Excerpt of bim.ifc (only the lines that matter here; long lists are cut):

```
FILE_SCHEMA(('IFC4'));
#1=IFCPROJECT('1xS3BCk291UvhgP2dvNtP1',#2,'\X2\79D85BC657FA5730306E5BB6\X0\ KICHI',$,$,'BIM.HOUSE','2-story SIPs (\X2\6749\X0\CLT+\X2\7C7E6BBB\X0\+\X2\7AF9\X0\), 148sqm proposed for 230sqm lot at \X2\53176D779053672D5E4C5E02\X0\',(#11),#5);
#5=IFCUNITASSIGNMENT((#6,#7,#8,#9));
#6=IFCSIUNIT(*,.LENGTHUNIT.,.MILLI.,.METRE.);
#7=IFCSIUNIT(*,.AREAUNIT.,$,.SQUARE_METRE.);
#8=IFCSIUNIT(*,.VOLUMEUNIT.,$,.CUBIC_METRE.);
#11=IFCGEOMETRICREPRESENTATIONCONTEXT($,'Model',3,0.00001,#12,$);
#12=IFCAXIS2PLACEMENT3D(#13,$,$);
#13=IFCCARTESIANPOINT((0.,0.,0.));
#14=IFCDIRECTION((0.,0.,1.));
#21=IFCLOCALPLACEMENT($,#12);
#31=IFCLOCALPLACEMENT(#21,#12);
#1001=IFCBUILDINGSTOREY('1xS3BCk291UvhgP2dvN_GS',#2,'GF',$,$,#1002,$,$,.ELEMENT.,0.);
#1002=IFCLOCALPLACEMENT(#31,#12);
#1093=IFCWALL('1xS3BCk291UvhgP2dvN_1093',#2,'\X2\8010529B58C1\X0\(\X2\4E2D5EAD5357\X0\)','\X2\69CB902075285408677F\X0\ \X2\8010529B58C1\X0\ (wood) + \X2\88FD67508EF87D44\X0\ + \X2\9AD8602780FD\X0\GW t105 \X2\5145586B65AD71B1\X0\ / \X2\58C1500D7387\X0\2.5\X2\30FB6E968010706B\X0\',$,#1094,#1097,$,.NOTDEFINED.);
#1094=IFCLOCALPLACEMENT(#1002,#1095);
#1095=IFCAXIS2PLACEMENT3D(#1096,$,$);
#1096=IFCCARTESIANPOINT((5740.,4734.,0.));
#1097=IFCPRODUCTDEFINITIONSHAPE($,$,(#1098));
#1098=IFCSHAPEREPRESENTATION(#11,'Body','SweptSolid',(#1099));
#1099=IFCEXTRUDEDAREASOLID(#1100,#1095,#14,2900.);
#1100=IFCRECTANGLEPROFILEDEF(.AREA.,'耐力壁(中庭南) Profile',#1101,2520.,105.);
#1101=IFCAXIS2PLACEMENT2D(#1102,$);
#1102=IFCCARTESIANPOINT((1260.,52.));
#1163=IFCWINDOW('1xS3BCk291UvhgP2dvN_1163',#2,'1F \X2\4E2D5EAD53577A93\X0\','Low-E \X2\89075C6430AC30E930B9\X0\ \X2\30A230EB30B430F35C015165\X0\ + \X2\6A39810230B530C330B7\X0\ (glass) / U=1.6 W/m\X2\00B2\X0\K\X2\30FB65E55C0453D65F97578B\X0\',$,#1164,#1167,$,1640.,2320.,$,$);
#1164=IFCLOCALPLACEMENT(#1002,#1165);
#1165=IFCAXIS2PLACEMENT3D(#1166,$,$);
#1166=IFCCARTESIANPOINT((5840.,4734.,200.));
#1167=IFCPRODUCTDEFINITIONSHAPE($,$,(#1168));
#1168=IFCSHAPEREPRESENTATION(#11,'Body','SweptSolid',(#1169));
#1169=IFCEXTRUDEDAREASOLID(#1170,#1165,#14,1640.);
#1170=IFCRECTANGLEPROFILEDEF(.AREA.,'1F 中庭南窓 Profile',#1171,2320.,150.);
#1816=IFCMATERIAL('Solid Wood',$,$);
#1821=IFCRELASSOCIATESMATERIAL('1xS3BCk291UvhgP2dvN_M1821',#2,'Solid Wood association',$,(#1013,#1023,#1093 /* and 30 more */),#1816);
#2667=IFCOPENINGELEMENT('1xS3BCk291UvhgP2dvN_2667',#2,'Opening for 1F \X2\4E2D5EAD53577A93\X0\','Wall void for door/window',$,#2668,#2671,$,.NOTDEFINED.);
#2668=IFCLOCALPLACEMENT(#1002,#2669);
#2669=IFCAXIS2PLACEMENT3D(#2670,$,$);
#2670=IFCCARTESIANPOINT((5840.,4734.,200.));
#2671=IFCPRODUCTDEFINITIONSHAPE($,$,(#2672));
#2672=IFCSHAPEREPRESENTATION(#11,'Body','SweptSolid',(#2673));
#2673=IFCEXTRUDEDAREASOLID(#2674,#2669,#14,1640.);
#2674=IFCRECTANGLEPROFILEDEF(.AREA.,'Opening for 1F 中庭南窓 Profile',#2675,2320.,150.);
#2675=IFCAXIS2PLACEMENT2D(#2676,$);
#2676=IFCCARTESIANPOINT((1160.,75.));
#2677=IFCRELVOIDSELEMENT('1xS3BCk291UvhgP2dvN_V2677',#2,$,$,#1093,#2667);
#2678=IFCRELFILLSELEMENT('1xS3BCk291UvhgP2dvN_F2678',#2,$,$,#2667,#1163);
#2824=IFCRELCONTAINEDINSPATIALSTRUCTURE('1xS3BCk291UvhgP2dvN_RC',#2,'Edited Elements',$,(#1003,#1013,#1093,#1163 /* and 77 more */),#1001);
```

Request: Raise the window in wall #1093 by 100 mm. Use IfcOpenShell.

```python
import numpy as np
import ifcopenshell
import ifcopenshell.api.geometry
import ifcopenshell.util.placement
import ifcopenshell.util.unit

model = ifcopenshell.open("bim.ifc")
unit_scale = ifcopenshell.util.unit.calculate_unit_scale(model)

window = model.by_guid("1xS3BCk291UvhgP2dvN_1163")
opening = window.FillsVoids[0].RelatingOpeningElement
dz = 0.1 / unit_scale

shift = np.array([0.0, 0.0, dz])
# The window is not placed relative to its opening, so move both.
for product in (opening, window):
    matrix = ifcopenshell.util.placement.get_local_placement(product.ObjectPlacement)
    matrix[:3, 3] += shift
    ifcopenshell.api.geometry.edit_object_placement(model, product=product, matrix=matrix, is_si=False)

print(f"moved by {dz * unit_scale:+.3f} m")

model.write("bim_edited.ifc")
```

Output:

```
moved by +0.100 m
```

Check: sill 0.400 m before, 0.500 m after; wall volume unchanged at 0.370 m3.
